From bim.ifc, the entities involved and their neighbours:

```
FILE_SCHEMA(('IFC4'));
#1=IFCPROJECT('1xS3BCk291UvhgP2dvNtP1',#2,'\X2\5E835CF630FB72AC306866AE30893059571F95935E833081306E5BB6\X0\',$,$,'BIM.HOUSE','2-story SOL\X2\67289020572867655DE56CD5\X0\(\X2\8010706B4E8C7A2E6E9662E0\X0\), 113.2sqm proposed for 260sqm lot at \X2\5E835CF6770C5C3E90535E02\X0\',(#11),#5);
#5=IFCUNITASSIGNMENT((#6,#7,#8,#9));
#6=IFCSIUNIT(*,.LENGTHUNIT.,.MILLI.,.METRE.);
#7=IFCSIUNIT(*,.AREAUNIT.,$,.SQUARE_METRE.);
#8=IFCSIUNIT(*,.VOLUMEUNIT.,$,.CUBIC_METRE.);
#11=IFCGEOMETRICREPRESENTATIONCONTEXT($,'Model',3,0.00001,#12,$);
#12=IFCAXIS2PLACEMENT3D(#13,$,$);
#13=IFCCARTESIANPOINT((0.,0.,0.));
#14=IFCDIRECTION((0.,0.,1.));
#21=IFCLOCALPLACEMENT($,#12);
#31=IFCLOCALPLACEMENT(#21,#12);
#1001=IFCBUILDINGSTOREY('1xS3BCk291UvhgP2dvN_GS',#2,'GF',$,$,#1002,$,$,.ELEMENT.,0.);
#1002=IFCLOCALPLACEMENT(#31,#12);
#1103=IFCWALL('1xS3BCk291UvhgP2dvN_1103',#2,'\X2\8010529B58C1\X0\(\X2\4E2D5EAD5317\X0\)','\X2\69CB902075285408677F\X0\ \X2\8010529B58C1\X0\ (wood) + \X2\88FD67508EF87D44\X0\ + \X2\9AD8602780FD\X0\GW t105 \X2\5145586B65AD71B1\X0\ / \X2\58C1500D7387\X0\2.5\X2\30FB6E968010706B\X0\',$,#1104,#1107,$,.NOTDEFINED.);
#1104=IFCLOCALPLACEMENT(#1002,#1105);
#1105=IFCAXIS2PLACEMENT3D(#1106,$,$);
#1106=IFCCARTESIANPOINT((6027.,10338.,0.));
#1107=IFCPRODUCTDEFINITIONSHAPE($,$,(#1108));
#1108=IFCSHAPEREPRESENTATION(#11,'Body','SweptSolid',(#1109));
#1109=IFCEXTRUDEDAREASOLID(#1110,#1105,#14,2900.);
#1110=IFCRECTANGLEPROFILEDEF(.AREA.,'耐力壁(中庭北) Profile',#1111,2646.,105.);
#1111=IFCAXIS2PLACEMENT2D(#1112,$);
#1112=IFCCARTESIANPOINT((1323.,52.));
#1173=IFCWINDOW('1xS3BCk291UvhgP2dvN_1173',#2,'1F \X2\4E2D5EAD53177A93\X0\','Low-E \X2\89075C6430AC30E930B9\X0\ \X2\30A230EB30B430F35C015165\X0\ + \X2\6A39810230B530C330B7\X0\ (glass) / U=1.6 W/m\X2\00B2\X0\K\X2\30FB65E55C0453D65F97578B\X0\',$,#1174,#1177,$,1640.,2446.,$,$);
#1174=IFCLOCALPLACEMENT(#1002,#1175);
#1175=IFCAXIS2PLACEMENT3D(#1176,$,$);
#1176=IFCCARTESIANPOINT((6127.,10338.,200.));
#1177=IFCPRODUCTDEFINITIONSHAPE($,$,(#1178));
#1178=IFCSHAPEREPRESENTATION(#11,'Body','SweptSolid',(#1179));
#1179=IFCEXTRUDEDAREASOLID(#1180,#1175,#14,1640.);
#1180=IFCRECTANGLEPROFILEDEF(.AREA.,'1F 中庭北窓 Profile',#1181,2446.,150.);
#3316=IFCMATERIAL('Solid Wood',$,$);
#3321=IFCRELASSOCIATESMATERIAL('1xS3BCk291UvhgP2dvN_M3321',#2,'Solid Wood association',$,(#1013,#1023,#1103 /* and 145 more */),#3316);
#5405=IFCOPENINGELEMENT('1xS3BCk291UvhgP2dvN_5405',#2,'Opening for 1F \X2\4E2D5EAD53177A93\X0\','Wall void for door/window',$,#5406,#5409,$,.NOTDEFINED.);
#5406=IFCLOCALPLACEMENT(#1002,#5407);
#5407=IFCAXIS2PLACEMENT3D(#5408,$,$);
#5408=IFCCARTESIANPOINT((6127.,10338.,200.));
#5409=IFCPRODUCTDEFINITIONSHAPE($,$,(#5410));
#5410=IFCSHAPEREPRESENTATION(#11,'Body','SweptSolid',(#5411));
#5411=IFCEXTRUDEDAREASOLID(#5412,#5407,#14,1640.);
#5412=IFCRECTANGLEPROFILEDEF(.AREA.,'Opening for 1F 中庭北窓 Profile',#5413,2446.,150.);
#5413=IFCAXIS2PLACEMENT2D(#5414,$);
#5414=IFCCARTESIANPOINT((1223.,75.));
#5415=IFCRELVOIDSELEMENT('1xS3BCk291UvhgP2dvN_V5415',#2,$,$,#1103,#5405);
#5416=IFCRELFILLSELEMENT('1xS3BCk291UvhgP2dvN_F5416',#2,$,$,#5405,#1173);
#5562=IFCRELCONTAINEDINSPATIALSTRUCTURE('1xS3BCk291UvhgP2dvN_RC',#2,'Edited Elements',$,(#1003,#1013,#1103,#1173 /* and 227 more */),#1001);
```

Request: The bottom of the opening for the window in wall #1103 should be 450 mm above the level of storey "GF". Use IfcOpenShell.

```python
import numpy as np
import ifcopenshell
import ifcopenshell.api.geometry
import ifcopenshell.geom
import ifcopenshell.util.element
import ifcopenshell.util.placement
import ifcopenshell.util.shape
import ifcopenshell.util.unit

model = ifcopenshell.open("bim.ifc")
unit_scale = ifcopenshell.util.unit.calculate_unit_scale(model)

window = model.by_id(1173)
opening = window.FillsVoids[0].RelatingOpeningElement
storey = ifcopenshell.util.element.get_container(window, ifc_class="IfcBuildingStorey")
level = ifcopenshell.util.placement.get_local_placement(storey.ObjectPlacement)[2, 3]

# The opening's origin need not be at the sill, so measure its lowest point.
shape = ifcopenshell.geom.create_shape(ifcopenshell.geom.settings(), opening)
bottom = ifcopenshell.util.shape.get_shape_bottom_elevation(shape, shape.geometry) / unit_scale
dz = level + 0.45 / unit_scale - bottom

shift = np.array([0.0, 0.0, dz])
# The window is not placed relative to its opening, so move both.
for product in (opening, window):
    matrix = ifcopenshell.util.placement.get_local_placement(product.ObjectPlacement)
    matrix[:3, 3] += shift
    ifcopenshell.api.geometry.edit_object_placement(model, product=product, matrix=matrix, is_si=False)

print(f"moved by {dz * unit_scale:+.3f} m")

model.write("bim_updated.ifc")
```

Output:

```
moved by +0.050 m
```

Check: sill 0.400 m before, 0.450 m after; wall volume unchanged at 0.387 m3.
